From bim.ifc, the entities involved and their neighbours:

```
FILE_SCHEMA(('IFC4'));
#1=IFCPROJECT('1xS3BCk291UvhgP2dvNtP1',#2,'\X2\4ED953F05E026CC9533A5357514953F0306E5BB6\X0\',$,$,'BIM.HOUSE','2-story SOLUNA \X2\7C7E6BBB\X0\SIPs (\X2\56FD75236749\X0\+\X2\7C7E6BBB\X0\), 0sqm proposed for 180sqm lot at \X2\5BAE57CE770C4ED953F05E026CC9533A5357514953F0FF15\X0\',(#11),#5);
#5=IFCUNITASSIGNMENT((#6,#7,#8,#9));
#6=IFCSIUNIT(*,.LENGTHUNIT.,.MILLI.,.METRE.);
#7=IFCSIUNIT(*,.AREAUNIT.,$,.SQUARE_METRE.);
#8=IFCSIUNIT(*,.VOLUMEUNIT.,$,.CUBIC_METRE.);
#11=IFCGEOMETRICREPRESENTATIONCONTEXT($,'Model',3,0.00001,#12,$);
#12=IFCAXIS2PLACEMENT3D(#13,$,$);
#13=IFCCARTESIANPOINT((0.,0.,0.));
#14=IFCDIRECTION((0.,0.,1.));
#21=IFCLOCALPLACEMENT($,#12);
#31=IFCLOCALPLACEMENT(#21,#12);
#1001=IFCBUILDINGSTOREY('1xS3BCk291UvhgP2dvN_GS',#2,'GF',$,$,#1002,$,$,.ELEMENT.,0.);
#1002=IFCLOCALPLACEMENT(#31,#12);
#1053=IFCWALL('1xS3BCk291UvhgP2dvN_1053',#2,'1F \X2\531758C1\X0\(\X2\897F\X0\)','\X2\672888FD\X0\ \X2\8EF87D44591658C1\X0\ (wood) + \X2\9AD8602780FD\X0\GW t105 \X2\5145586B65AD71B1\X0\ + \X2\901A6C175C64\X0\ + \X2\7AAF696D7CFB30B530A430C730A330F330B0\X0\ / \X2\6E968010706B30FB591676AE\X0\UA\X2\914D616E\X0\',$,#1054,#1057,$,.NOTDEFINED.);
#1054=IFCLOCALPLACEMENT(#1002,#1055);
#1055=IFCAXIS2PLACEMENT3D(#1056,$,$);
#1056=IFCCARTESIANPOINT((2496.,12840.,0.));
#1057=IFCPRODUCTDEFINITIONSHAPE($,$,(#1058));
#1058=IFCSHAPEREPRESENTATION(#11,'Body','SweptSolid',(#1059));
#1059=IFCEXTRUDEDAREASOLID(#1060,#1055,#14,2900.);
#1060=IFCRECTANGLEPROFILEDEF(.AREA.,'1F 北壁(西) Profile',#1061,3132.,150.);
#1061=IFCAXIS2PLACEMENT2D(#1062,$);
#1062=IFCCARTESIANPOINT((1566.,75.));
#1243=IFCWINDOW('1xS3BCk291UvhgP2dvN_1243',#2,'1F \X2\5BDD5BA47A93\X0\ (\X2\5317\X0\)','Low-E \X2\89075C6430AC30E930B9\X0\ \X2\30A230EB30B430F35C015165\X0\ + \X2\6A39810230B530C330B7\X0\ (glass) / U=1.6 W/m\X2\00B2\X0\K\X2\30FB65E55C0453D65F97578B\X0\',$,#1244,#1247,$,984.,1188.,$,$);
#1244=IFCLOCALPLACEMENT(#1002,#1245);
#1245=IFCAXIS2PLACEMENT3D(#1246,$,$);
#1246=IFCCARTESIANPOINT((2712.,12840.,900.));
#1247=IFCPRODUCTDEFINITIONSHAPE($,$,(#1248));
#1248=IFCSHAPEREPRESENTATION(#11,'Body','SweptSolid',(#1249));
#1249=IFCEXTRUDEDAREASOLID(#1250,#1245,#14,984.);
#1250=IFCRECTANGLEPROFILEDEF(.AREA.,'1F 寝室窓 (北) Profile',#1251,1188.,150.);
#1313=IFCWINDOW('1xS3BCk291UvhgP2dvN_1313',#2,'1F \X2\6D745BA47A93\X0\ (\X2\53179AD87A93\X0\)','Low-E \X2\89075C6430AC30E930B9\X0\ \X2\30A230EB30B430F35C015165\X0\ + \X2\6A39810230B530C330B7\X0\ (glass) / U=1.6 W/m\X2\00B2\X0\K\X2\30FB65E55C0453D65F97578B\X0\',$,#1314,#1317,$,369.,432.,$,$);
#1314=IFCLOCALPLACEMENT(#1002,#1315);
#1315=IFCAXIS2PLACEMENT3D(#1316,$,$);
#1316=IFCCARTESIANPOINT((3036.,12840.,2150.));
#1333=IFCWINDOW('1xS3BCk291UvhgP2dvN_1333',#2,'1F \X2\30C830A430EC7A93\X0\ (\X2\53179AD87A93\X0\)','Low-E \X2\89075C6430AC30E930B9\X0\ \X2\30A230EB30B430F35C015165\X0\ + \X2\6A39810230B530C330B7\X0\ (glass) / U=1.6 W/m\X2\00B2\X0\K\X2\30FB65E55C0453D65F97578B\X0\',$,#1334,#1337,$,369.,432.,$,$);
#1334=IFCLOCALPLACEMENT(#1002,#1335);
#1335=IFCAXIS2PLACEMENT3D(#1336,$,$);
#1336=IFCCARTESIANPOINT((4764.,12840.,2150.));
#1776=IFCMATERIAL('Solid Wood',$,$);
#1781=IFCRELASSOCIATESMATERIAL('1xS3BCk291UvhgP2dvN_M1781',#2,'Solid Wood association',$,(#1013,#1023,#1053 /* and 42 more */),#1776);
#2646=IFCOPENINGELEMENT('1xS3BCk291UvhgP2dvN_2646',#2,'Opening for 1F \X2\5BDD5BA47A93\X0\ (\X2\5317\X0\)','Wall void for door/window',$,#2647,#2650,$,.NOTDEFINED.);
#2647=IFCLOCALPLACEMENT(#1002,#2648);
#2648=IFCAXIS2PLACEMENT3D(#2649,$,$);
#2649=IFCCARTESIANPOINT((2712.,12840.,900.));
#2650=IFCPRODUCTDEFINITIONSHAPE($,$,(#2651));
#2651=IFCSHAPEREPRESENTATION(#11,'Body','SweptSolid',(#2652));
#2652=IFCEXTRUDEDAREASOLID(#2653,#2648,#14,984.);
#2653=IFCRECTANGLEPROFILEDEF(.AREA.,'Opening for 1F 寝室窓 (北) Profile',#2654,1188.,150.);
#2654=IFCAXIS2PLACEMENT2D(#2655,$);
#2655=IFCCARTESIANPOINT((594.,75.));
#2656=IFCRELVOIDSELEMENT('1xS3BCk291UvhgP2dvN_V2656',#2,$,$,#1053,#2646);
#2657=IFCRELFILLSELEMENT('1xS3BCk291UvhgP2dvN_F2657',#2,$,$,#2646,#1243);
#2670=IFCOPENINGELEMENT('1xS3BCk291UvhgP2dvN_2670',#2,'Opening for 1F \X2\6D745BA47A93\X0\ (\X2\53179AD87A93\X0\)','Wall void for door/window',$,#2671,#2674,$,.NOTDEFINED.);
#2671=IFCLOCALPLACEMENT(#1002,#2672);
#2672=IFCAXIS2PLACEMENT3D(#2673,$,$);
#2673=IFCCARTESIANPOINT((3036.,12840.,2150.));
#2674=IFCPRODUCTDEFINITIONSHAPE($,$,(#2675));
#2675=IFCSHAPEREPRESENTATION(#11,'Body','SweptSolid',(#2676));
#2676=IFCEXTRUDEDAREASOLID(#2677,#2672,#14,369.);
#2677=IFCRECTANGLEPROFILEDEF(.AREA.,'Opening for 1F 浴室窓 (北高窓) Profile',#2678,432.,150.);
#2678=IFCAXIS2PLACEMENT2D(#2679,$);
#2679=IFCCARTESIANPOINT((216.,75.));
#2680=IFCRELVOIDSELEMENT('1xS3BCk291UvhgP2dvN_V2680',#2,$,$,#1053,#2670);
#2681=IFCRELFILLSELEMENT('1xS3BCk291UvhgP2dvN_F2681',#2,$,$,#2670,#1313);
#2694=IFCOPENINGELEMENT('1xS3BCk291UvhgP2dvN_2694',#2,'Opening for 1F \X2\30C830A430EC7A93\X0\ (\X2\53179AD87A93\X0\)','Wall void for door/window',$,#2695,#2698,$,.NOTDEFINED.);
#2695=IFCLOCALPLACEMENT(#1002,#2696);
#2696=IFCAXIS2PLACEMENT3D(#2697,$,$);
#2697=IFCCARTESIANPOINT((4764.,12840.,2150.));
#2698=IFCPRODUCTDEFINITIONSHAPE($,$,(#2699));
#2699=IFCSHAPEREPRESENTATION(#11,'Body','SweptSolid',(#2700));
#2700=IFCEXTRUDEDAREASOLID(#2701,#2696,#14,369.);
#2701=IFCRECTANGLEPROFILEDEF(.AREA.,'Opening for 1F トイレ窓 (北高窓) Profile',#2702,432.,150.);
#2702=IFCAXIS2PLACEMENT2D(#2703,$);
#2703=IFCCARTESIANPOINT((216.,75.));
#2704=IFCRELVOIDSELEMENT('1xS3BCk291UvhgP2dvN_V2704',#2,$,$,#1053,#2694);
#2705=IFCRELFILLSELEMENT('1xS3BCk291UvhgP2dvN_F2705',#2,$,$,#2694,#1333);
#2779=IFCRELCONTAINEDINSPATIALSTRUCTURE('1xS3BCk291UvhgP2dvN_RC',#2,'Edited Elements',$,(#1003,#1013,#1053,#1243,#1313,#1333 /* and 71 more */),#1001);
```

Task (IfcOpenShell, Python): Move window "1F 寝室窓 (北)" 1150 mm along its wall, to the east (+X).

```python
import ifcopenshell
import ifcopenshell.api.geometry
import ifcopenshell.util.placement

model = ifcopenshell.open("bim.ifc")

window = model.by_id(1243)
opening = window.FillsVoids[0].RelatingOpeningElement
wall = opening.VoidsElements[0].RelatingBuildingElement

wall_matrix = ifcopenshell.util.placement.get_local_placement(wall.ObjectPlacement)
shift = wall_matrix[:3, 0] * 1150.0
before = ifcopenshell.util.placement.get_local_placement(window.ObjectPlacement)[:3, 3].copy()

# The window is not placed relative to its opening, so move both.
for product in (opening, window):
    matrix = ifcopenshell.util.placement.get_local_placement(product.ObjectPlacement)
    matrix[:3, 3] += shift
    ifcopenshell.api.geometry.edit_object_placement(model, product=product, matrix=matrix, is_si=False)

after = ifcopenshell.util.placement.get_local_placement(window.ObjectPlacement)[:3, 3]
print("window moved by", (after - before).round(3) + 0.0)

model.write("bim-out.ifc")
```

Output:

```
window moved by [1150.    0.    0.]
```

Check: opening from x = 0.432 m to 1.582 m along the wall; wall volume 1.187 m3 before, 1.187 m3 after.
